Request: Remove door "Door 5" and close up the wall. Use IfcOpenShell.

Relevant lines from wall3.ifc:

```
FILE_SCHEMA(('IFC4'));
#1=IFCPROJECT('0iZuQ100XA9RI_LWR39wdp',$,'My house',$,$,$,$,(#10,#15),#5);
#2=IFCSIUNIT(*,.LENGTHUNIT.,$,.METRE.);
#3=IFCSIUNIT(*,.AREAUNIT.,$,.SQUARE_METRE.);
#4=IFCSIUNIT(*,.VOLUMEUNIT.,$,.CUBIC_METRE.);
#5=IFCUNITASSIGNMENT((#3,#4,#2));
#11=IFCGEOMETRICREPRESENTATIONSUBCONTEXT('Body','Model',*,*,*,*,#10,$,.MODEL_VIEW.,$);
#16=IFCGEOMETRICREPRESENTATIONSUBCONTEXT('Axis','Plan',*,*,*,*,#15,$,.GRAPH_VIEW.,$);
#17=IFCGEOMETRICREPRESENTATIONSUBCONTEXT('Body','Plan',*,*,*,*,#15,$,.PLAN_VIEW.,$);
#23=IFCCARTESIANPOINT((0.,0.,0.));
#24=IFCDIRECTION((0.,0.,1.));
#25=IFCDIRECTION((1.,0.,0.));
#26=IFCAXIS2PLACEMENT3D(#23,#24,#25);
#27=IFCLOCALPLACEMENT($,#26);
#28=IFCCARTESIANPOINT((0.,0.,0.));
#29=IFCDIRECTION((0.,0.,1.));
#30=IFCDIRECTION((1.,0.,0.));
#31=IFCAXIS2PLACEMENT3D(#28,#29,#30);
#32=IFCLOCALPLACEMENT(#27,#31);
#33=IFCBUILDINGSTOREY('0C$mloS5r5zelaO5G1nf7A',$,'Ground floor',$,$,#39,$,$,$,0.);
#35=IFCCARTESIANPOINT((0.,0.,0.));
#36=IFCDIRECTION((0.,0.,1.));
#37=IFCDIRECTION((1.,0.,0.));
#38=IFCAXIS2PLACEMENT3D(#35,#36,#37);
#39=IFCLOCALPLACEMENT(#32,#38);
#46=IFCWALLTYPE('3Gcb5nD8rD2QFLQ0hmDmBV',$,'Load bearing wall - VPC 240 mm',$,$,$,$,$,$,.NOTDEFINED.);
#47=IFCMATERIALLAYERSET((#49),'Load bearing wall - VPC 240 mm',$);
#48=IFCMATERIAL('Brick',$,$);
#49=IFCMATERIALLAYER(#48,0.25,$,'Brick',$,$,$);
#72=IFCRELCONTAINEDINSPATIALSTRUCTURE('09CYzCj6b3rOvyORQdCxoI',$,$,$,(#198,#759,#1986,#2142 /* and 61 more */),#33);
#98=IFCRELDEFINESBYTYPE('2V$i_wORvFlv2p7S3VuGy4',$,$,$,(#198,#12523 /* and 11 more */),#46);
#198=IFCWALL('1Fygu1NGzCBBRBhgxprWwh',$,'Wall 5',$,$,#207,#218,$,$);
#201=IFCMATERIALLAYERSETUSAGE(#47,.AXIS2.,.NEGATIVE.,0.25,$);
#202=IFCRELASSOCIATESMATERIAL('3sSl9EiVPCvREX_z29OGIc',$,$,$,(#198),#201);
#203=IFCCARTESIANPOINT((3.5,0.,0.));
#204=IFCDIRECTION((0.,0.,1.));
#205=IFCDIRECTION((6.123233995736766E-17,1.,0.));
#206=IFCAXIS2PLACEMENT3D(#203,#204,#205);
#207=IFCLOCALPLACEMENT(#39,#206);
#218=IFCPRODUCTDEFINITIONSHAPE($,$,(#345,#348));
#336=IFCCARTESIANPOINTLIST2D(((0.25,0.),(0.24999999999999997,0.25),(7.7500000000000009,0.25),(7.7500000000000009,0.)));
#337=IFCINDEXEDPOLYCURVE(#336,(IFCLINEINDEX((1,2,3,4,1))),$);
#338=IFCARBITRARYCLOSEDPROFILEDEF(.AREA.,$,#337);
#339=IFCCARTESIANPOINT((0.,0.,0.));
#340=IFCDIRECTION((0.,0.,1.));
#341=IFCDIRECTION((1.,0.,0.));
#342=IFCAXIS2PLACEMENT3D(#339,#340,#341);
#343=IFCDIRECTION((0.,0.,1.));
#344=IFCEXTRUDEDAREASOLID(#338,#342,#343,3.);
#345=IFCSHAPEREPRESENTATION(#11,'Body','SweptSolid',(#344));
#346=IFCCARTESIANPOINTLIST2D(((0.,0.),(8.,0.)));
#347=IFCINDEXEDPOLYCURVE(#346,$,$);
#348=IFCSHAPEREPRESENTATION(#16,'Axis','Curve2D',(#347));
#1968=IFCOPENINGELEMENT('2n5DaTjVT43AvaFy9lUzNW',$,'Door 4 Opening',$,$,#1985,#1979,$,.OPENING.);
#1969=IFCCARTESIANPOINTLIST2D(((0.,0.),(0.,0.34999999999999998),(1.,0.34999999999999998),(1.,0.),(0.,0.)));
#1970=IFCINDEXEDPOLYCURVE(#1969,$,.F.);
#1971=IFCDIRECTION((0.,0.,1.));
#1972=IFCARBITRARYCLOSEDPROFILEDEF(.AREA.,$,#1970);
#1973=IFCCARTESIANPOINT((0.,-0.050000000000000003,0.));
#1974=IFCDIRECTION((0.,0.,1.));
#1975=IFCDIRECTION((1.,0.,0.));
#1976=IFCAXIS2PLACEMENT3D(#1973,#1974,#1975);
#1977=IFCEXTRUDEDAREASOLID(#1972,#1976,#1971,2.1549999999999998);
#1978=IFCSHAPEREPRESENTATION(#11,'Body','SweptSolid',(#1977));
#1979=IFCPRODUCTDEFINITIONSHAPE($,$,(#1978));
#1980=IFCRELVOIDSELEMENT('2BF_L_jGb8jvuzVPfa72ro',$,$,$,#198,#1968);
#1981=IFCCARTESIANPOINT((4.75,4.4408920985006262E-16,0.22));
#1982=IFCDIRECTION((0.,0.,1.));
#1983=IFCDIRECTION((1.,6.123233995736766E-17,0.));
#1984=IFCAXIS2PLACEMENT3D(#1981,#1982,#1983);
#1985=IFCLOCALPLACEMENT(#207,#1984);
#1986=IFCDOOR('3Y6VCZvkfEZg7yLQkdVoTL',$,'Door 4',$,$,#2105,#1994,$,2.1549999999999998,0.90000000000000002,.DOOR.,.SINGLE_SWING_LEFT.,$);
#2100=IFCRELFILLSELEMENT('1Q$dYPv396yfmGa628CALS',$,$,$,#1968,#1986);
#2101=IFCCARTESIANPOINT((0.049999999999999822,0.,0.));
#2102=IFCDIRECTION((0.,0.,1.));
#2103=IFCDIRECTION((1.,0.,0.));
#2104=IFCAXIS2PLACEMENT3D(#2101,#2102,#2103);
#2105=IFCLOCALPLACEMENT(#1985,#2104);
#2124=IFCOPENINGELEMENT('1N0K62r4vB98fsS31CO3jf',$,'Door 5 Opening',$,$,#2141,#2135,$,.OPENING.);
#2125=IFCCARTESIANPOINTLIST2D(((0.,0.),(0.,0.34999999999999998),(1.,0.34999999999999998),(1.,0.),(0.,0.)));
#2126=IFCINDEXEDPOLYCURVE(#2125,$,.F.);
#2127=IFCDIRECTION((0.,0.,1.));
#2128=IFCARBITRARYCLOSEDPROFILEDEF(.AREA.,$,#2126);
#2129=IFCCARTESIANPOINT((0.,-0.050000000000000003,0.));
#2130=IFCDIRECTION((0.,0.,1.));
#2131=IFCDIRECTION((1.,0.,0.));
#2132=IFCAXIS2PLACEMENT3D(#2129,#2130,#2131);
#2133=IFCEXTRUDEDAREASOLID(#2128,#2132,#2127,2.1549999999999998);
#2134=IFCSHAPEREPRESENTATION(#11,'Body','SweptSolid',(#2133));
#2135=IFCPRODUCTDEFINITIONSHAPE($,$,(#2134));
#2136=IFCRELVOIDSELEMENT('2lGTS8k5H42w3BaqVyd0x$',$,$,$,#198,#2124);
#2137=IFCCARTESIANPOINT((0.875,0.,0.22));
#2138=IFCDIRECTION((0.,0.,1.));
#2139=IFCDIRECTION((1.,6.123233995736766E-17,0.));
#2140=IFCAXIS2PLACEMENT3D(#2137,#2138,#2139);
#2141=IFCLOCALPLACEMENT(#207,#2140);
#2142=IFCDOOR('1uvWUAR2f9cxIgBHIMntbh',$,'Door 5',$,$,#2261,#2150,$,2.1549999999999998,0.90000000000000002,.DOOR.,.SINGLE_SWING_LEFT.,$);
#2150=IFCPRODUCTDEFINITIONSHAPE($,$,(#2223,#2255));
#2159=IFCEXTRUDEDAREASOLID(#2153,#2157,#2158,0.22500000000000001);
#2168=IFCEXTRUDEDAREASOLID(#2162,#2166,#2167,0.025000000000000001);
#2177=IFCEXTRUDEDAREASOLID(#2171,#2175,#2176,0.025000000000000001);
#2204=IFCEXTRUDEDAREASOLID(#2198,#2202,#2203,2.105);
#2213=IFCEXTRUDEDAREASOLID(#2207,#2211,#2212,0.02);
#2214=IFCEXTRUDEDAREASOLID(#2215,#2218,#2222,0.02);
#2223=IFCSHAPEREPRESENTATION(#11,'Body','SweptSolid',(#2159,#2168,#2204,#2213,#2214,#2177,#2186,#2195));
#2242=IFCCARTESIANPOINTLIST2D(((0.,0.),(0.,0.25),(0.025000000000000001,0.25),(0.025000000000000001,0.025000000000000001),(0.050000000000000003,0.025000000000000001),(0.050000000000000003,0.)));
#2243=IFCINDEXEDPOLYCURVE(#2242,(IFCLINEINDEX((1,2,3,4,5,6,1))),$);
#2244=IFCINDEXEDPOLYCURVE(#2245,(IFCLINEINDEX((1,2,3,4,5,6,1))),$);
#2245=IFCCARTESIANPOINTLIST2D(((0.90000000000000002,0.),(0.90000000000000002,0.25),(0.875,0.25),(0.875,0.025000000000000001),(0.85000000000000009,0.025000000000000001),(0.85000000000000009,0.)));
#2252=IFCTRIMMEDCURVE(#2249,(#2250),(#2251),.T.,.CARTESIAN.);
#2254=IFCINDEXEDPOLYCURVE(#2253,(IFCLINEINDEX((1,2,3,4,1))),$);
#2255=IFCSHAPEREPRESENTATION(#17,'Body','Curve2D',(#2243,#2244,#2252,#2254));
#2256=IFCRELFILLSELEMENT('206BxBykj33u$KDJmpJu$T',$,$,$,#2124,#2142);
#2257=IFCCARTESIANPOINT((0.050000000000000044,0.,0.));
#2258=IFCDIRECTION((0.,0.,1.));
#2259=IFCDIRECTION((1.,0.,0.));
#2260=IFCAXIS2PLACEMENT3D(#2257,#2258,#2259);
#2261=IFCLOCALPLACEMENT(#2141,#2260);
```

```python
import ifcopenshell
import ifcopenshell.api.feature
import ifcopenshell.api.root
import ifcopenshell.geom
import ifcopenshell.util.shape

model = ifcopenshell.open("wall3.ifc")
settings = ifcopenshell.geom.settings()


def volume(element):
    """Net volume in cubic metres, openings subtracted."""
    shape = ifcopenshell.geom.create_shape(settings, element)
    return ifcopenshell.util.shape.get_volume(shape.geometry)


door = model.by_guid("1uvWUAR2f9cxIgBHIMntbh")
opening = door.FillsVoids[0].RelatingOpeningElement
wall = opening.VoidsElements[0].RelatingBuildingElement
before = volume(wall)

ifcopenshell.api.root.remove_product(model, product=door)
ifcopenshell.api.feature.remove_feature(model, feature=opening)

after = volume(wall)

print(f"wall volume {before:.3f} -> {after:.3f} m3")

model.write("wall3_edited.ifc")
```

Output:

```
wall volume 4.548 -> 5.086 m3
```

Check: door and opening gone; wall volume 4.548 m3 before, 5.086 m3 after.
